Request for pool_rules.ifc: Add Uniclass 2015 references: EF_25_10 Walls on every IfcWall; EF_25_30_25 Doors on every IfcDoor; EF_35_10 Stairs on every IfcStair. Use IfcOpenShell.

First a look at what the model holds.

```python
import ifcopenshell

model = ifcopenshell.open("pool_rules.ifc")
print(model.schema)
print("classifications:", [c.Name for c in model.by_type("IfcClassification")])
for ifc_class in ("IfcDoor", "IfcRoof", "IfcStair", "IfcWall", "IfcWindow"):
    print(ifc_class, len(model.by_type(ifc_class)))
```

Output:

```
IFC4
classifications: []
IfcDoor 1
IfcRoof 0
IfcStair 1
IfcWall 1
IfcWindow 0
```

```python
import ifcopenshell
import ifcopenshell.api.classification

model = ifcopenshell.open("pool_rules.ifc")

system = ifcopenshell.api.classification.add_classification(model, classification="Uniclass 2015")

codes = {
    "IfcWall": ("EF_25_10", "Walls"),
    "IfcDoor": ("EF_25_30_25", "Doors"),
    "IfcStair": ("EF_35_10", "Stairs"),
}
for ifc_class, (code, name) in codes.items():
    products = model.by_type(ifc_class)
    ifcopenshell.api.classification.add_reference(
        model, products=products, classification=system, identification=code, name=name
    )
    print(code, len(products))

model.write("pool_rules_v2.ifc")
```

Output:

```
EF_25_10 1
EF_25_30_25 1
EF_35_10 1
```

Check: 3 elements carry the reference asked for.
